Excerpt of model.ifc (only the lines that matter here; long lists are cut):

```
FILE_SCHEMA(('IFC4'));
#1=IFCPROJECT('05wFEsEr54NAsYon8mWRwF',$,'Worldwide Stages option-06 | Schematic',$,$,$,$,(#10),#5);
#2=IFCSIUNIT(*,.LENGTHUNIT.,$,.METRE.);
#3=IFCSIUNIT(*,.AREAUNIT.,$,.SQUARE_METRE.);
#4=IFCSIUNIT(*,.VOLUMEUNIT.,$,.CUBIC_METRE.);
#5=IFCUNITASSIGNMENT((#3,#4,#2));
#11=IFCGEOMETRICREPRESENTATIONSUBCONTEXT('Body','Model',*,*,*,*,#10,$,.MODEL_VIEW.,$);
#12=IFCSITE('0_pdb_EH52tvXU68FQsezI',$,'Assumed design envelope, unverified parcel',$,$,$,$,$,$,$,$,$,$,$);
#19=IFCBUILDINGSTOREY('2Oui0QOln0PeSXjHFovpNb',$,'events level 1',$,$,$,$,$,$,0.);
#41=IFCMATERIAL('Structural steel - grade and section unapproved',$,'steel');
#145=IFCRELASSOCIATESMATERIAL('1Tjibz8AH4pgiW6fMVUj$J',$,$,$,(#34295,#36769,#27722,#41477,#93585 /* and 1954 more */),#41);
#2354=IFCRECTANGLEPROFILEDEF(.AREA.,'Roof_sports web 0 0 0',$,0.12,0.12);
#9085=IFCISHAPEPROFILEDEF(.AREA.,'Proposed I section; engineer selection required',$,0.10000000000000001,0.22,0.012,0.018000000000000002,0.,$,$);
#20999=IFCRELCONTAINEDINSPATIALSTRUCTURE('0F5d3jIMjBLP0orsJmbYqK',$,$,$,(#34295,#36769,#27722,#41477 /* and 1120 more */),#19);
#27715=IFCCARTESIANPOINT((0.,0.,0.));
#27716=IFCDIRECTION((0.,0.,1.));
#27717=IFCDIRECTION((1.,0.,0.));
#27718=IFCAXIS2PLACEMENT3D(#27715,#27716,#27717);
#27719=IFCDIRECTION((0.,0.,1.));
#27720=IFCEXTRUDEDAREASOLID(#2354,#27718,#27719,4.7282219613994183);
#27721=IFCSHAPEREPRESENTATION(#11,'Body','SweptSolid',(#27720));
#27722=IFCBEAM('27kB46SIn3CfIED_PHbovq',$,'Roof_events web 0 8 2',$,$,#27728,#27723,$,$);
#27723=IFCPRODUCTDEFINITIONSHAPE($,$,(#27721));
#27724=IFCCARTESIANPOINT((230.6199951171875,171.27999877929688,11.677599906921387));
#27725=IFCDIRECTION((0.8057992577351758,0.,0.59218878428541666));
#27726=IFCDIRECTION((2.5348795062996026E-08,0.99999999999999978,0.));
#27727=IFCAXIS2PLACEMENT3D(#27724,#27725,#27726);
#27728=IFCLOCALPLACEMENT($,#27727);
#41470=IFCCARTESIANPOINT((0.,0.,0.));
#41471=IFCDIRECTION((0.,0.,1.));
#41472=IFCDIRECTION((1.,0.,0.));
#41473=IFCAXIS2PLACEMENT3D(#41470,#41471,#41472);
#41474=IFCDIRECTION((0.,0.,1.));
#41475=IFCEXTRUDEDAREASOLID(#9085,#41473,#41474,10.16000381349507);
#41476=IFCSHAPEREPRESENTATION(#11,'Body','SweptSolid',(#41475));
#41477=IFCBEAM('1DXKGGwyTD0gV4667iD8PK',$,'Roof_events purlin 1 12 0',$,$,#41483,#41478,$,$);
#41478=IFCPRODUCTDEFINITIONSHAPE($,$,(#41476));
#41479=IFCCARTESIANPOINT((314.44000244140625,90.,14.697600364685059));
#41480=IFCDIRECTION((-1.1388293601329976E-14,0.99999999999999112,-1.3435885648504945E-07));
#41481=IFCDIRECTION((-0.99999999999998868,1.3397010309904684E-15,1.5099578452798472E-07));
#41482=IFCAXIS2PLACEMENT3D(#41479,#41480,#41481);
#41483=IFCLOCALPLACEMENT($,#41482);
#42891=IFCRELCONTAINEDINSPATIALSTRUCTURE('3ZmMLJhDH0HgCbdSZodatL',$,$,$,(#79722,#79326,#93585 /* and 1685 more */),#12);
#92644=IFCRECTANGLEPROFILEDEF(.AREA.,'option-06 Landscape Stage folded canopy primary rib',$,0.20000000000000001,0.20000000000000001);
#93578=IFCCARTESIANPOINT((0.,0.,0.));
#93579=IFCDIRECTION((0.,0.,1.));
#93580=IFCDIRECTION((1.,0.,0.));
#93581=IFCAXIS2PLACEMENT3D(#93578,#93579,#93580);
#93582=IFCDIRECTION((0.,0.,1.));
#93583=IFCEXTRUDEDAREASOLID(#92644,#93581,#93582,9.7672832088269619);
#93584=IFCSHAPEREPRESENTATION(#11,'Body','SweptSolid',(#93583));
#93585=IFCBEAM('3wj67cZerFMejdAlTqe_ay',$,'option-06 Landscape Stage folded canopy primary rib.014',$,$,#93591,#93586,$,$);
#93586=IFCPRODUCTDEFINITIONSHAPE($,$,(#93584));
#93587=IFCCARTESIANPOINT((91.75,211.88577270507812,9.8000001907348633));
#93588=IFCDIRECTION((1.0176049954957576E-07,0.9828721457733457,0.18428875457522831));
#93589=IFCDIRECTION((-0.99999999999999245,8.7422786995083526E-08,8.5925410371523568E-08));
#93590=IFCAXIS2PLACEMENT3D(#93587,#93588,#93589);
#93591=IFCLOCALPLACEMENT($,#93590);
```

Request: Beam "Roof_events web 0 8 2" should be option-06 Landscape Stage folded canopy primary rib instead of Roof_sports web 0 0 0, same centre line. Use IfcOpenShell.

```python
import ifcopenshell
import ifcopenshell.util.element
import ifcopenshell.util.representation

model = ifcopenshell.open("model.ifc")

member = model.by_guid("27kB46SIn3CfIED_PHbovq")
source = next(p for p in model.by_type("IfcRectangleProfileDef") if p.ProfileName == "option-06 Landscape Stage folded canopy primary rib")

body = ifcopenshell.util.representation.get_representation(member, "Model", "Body")
solid = body.Items[0]
old_profile = solid.SweptArea

# Copy the section's sizes but keep this member's own profile position.
profile = ifcopenshell.util.element.copy(model, source)
profile.Position = old_profile.Position
solid.SweptArea = profile
if not model.get_total_inverses(old_profile):
    ifcopenshell.util.element.remove_deep2(model, old_profile)

print(solid.SweptArea)

model.write("model_rev.ifc")
```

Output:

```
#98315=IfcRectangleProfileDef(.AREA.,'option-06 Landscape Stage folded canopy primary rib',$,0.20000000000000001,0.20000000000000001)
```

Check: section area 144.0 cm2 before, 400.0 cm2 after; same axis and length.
